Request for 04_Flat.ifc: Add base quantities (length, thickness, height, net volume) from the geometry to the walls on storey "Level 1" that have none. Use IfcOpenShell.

First a look at what the model holds.

```python
import ifcopenshell
import ifcopenshell.util.element
import ifcopenshell.util.unit

model = ifcopenshell.open("04_Flat.ifc")
print(model.schema)
for unit_type in ("LENGTHUNIT", "AREAUNIT", "VOLUMEUNIT"):
    print(unit_type, ifcopenshell.util.unit.calculate_unit_scale(model, unit_type))
storey = next(s for s in model.by_type("IfcBuildingStorey") if s.Name == "Level 1")
walls = [e for e in ifcopenshell.util.element.get_decomposition(storey) if e.is_a("IfcWall")]
for e in sorted(walls, key=lambda e: e.id()):
    print(e.id(), e.is_a(), e.Name, list(ifcopenshell.util.element.get_psets(e, qtos_only=True)), sep=" | ")
```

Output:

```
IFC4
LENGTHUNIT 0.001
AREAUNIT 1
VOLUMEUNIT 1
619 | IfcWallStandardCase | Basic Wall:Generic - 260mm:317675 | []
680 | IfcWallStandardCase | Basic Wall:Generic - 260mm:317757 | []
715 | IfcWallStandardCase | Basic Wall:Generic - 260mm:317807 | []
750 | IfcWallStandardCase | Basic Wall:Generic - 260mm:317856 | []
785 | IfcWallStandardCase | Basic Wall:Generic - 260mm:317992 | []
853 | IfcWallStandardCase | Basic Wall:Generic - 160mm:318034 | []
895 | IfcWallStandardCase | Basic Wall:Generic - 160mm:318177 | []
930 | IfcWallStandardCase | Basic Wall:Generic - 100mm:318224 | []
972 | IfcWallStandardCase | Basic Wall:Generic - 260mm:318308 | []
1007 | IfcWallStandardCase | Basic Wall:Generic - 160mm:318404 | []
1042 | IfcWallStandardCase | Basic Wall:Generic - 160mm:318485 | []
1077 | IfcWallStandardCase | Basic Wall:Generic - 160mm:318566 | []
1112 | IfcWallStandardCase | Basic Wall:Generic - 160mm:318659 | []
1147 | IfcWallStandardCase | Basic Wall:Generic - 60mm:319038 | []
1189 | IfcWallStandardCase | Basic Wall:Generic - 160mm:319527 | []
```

```python
import ifcopenshell
import ifcopenshell.api.pset
import ifcopenshell.geom
import ifcopenshell.util.element
import ifcopenshell.util.shape
import ifcopenshell.util.unit

model = ifcopenshell.open("04_Flat.ifc")
unit_scale = ifcopenshell.util.unit.calculate_unit_scale(model)
volume_scale = ifcopenshell.util.unit.calculate_unit_scale(model, "VOLUMEUNIT")
settings = ifcopenshell.geom.settings()

storey = next(s for s in model.by_type("IfcBuildingStorey") if s.Name == "Level 1")
walls = [e for e in ifcopenshell.util.element.get_decomposition(storey) if e.is_a("IfcWall")]

for e in sorted(walls, key=lambda e: e.id()):
    if ifcopenshell.util.element.get_psets(e, qtos_only=True, should_inherit=False):
        continue
    # Geometry comes back in metres, in the element's own axes.
    shape = ifcopenshell.geom.create_shape(settings, e)
    values = {
        "Length": ifcopenshell.util.shape.get_x(shape.geometry) / unit_scale,
        "Width": ifcopenshell.util.shape.get_y(shape.geometry) / unit_scale,
        "Height": ifcopenshell.util.shape.get_z(shape.geometry) / unit_scale,
        "NetVolume": ifcopenshell.util.shape.get_volume(shape.geometry) / volume_scale,
    }
    qto = ifcopenshell.api.pset.add_qto(model, product=e, name="Qto_WallBaseQuantities")
    ifcopenshell.api.pset.edit_qto(model, qto=qto, properties=values)
    print(e.id(), {k: round(v, 3) for k, v in values.items()})

model.write("04_Flat_rev.ifc")
```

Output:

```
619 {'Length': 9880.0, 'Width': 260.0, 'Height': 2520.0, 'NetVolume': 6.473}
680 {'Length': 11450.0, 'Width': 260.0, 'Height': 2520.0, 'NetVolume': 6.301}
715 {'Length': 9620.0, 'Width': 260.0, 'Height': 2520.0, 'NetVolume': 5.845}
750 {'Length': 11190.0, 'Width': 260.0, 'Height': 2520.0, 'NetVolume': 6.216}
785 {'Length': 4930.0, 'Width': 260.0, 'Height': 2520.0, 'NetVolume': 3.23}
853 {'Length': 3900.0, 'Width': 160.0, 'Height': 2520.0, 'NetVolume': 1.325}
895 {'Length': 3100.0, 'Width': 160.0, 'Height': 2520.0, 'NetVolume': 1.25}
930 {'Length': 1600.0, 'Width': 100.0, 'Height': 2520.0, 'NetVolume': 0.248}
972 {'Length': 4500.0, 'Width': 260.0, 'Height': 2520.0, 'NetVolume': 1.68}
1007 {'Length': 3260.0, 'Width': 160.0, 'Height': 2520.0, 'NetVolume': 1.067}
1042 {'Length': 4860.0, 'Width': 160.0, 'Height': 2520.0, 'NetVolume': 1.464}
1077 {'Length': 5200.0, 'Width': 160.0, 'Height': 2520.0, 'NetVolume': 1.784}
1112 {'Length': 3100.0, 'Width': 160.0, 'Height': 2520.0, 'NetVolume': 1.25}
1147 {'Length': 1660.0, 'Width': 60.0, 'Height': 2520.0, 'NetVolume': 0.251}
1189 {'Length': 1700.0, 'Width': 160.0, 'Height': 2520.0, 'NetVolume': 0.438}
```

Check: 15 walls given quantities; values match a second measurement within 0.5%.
